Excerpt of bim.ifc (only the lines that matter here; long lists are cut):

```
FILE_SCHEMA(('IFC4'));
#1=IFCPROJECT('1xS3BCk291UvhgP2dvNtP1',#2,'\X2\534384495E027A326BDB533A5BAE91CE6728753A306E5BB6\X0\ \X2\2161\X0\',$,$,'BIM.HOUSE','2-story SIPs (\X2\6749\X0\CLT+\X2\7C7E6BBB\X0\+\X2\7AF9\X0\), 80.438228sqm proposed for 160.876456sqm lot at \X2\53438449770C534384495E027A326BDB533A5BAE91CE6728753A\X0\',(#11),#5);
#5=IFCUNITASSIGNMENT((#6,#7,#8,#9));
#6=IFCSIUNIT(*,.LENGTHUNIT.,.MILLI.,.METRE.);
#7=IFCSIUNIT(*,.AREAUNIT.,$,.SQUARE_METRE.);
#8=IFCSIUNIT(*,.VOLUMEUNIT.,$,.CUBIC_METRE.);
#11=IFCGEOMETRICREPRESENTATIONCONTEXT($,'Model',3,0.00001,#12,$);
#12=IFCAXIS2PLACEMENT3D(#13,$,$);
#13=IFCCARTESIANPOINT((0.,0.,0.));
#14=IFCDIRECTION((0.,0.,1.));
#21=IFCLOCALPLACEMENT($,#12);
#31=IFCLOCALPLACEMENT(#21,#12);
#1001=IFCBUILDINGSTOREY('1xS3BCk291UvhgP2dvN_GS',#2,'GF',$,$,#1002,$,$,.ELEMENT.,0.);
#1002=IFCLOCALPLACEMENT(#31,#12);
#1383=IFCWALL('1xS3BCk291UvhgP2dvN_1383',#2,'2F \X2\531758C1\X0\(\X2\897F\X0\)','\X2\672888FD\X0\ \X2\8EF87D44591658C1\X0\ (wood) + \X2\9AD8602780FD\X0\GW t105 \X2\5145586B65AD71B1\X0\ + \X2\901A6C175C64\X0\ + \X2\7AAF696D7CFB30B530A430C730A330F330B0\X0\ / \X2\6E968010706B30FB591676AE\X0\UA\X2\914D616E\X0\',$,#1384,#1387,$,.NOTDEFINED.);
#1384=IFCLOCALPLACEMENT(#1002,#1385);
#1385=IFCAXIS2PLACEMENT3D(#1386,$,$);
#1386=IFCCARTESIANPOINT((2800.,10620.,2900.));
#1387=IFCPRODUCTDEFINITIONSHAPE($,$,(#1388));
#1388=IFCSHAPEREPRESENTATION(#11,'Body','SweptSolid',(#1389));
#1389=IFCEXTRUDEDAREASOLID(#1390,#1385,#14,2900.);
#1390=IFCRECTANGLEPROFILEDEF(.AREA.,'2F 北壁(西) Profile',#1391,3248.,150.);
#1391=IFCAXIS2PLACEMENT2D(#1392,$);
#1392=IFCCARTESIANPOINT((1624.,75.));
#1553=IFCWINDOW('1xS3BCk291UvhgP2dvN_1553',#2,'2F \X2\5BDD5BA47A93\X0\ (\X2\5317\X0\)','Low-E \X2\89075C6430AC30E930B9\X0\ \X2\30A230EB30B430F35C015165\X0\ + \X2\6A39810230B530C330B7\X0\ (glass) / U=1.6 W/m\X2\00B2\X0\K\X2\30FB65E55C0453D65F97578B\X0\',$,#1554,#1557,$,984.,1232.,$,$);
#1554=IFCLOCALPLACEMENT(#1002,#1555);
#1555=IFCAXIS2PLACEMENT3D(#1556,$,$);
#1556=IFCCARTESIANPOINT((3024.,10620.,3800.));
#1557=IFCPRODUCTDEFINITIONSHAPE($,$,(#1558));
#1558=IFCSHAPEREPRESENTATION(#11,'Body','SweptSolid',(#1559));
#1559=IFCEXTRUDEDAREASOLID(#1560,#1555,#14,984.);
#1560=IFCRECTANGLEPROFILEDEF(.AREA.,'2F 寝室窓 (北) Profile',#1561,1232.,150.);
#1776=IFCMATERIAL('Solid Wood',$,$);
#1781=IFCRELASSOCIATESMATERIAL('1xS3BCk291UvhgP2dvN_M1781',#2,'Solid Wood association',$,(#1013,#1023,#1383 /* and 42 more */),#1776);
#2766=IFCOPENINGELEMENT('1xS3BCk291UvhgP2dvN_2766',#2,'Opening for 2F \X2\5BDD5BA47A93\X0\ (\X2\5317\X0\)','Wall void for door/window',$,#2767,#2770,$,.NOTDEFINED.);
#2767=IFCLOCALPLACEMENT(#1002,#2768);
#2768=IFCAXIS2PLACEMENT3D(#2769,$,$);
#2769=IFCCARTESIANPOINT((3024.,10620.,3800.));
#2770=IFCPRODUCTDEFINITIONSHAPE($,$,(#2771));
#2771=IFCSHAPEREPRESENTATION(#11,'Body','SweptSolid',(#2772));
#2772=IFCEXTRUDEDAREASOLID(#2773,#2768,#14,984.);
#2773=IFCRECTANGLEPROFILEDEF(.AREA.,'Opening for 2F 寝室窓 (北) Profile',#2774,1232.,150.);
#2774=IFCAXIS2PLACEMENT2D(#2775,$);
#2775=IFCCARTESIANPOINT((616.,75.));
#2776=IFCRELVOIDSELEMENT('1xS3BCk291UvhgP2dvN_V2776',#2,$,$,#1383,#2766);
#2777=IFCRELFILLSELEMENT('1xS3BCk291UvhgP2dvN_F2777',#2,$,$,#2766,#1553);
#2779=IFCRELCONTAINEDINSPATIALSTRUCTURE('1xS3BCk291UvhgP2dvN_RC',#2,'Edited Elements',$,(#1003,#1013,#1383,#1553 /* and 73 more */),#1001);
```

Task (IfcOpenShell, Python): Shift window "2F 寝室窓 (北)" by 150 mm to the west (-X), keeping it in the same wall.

```python
import ifcopenshell
import ifcopenshell.api.geometry
import ifcopenshell.util.placement

model = ifcopenshell.open("bim.ifc")

window = model.by_guid("1xS3BCk291UvhgP2dvN_1553")
opening = window.FillsVoids[0].RelatingOpeningElement
wall = opening.VoidsElements[0].RelatingBuildingElement

wall_matrix = ifcopenshell.util.placement.get_local_placement(wall.ObjectPlacement)
shift = wall_matrix[:3, 0] * -150.0
before = ifcopenshell.util.placement.get_local_placement(window.ObjectPlacement)[:3, 3].copy()

# The window is not placed relative to its opening, so move both.
for product in (opening, window):
    matrix = ifcopenshell.util.placement.get_local_placement(product.ObjectPlacement)
    matrix[:3, 3] += shift
    ifcopenshell.api.geometry.edit_object_placement(model, product=product, matrix=matrix, is_si=False)

after = ifcopenshell.util.placement.get_local_placement(window.ObjectPlacement)[:3, 3]
print("window moved by", (after - before).round(3) + 0.0)

model.write("bim_updated.ifc")
```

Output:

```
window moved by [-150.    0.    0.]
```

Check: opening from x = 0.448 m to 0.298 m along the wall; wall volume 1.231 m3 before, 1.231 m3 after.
